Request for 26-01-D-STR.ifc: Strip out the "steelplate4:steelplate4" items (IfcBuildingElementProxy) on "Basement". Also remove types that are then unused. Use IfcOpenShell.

First a look at what the model holds.

```python
import ifcopenshell
import ifcopenshell.util.element

model = ifcopenshell.open("26-01-D-STR.ifc")
print(model.schema)
storey = next(s for s in model.by_type("IfcBuildingStorey") if s.Name == "Basement")
proxies = [e for e in ifcopenshell.util.element.get_decomposition(storey) if e.is_a("IfcBuildingElementProxy")]
seen = {}
for e in proxies:
    element_type = ifcopenshell.util.element.get_type(e)
    name = element_type.Name if element_type not in (None, e) else None
    seen[name] = seen.get(name, 0) + 1
for name, count in sorted(seen.items(), key=str):
    print(count, "x", name)
```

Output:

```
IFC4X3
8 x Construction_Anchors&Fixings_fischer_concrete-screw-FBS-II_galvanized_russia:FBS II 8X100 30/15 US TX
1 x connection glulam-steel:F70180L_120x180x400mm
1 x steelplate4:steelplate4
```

```python
import ifcopenshell
import ifcopenshell.api.root
import ifcopenshell.util.element

model = ifcopenshell.open("26-01-D-STR.ifc")

storey = next(s for s in model.by_type("IfcBuildingStorey") if s.Name == "Basement")
proxies = [e for e in ifcopenshell.util.element.get_decomposition(storey) if e.is_a("IfcBuildingElementProxy")]
targets = [e for e in proxies if (t := ifcopenshell.util.element.get_type(e)) not in (None, e) and t.Name == "steelplate4:steelplate4"]
types = {ifcopenshell.util.element.get_type(e) for e in targets} - {None, *targets}

for e in targets:
    ifcopenshell.api.root.remove_product(model, product=e)
print(len(targets), "removed")

unused = [t for t in types if not ifcopenshell.util.element.get_types(t)]
for t in unused:
    ifcopenshell.api.root.remove_product(model, product=t)
print(len(unused), "unused types removed")

model.write("26-01-D-STR_edited.ifc")
```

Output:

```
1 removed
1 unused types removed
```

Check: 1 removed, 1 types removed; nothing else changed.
